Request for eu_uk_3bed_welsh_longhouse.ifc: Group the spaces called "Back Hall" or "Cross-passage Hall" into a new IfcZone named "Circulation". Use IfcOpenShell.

First a look at what the model holds.

```python
import ifcopenshell

model = ifcopenshell.open("eu_uk_3bed_welsh_longhouse.ifc")
print(model.schema)
seen = {}
for space in model.by_type("IfcSpace"):
    seen[space.LongName] = seen.get(space.LongName, 0) + 1
for name, count in sorted(seen.items(), key=str):
    print(count, "x", name)
print("zones:", [z.Name for z in model.by_type("IfcZone")][:20])
```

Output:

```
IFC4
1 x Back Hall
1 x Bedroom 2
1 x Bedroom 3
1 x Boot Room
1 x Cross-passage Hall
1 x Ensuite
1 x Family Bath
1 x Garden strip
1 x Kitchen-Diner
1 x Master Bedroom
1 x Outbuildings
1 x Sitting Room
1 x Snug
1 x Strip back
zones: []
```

```python
import ifcopenshell
import ifcopenshell.api.group
import ifcopenshell.api.root

model = ifcopenshell.open("eu_uk_3bed_welsh_longhouse.ifc")

names = {"Back Hall", "Cross-passage Hall"}
spaces = [s for s in model.by_type("IfcSpace") if s.LongName in names]

zone = ifcopenshell.api.root.create_entity(model, ifc_class="IfcZone", name="Circulation")
ifcopenshell.api.group.assign_group(model, products=spaces, group=zone)
print(len(spaces), "spaces in", zone.Name)

model.write("eu_uk_3bed_welsh_longhouse-out.ifc")
```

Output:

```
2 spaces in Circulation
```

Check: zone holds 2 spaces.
